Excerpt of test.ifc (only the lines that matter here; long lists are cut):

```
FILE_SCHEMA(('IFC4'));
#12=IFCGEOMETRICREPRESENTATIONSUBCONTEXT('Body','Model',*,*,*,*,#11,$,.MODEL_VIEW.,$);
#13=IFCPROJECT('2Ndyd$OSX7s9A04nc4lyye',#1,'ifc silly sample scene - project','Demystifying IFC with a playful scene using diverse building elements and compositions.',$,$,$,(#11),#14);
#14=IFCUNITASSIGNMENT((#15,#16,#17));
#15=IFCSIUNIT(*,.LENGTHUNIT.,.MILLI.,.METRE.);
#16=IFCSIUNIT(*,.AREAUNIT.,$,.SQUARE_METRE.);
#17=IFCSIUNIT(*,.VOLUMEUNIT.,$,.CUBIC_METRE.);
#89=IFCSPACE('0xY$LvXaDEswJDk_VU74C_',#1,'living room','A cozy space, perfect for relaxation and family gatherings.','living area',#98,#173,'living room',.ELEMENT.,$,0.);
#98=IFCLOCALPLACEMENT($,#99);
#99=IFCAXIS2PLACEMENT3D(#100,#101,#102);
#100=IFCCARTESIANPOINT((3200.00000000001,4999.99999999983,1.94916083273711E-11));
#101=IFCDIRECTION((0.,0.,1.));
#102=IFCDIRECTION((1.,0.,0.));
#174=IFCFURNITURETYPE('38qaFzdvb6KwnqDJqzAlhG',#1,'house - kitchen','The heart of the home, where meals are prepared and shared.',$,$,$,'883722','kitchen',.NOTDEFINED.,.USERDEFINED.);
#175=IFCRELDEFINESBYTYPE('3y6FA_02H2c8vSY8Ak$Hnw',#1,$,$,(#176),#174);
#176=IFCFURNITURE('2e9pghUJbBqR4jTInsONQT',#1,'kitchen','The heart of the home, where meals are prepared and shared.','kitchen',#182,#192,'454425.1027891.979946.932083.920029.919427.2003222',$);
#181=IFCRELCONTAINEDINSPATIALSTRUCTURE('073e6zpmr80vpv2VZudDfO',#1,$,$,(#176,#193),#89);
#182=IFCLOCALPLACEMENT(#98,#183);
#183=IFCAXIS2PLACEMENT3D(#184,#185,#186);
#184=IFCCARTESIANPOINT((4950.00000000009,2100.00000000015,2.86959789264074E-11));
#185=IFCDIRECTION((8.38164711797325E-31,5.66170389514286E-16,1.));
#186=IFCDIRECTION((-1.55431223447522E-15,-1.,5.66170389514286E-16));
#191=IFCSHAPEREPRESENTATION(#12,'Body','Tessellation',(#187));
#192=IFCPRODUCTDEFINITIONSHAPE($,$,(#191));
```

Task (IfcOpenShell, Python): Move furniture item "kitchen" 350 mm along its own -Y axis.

```python
import ifcopenshell
import ifcopenshell.api.geometry
import ifcopenshell.util.placement
import ifcopenshell.util.unit

model = ifcopenshell.open("test.ifc")
unit_scale = ifcopenshell.util.unit.calculate_unit_scale(model)

item = model.by_guid("2e9pghUJbBqR4jTInsONQT")
matrix = ifcopenshell.util.placement.get_local_placement(item.ObjectPlacement)
matrix[:3, 3] -= matrix[:3, 1] * 0.35 / unit_scale
ifcopenshell.api.geometry.edit_object_placement(model, product=item, matrix=matrix, is_si=False)

print(ifcopenshell.util.placement.get_local_placement(item.ObjectPlacement).round(3) + 0.0)

model.write("test_v2.ifc")
```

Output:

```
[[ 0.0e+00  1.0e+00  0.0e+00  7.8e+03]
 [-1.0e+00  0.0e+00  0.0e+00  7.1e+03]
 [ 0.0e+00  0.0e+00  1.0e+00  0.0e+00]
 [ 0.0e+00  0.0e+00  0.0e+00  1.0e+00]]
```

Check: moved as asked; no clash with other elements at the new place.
